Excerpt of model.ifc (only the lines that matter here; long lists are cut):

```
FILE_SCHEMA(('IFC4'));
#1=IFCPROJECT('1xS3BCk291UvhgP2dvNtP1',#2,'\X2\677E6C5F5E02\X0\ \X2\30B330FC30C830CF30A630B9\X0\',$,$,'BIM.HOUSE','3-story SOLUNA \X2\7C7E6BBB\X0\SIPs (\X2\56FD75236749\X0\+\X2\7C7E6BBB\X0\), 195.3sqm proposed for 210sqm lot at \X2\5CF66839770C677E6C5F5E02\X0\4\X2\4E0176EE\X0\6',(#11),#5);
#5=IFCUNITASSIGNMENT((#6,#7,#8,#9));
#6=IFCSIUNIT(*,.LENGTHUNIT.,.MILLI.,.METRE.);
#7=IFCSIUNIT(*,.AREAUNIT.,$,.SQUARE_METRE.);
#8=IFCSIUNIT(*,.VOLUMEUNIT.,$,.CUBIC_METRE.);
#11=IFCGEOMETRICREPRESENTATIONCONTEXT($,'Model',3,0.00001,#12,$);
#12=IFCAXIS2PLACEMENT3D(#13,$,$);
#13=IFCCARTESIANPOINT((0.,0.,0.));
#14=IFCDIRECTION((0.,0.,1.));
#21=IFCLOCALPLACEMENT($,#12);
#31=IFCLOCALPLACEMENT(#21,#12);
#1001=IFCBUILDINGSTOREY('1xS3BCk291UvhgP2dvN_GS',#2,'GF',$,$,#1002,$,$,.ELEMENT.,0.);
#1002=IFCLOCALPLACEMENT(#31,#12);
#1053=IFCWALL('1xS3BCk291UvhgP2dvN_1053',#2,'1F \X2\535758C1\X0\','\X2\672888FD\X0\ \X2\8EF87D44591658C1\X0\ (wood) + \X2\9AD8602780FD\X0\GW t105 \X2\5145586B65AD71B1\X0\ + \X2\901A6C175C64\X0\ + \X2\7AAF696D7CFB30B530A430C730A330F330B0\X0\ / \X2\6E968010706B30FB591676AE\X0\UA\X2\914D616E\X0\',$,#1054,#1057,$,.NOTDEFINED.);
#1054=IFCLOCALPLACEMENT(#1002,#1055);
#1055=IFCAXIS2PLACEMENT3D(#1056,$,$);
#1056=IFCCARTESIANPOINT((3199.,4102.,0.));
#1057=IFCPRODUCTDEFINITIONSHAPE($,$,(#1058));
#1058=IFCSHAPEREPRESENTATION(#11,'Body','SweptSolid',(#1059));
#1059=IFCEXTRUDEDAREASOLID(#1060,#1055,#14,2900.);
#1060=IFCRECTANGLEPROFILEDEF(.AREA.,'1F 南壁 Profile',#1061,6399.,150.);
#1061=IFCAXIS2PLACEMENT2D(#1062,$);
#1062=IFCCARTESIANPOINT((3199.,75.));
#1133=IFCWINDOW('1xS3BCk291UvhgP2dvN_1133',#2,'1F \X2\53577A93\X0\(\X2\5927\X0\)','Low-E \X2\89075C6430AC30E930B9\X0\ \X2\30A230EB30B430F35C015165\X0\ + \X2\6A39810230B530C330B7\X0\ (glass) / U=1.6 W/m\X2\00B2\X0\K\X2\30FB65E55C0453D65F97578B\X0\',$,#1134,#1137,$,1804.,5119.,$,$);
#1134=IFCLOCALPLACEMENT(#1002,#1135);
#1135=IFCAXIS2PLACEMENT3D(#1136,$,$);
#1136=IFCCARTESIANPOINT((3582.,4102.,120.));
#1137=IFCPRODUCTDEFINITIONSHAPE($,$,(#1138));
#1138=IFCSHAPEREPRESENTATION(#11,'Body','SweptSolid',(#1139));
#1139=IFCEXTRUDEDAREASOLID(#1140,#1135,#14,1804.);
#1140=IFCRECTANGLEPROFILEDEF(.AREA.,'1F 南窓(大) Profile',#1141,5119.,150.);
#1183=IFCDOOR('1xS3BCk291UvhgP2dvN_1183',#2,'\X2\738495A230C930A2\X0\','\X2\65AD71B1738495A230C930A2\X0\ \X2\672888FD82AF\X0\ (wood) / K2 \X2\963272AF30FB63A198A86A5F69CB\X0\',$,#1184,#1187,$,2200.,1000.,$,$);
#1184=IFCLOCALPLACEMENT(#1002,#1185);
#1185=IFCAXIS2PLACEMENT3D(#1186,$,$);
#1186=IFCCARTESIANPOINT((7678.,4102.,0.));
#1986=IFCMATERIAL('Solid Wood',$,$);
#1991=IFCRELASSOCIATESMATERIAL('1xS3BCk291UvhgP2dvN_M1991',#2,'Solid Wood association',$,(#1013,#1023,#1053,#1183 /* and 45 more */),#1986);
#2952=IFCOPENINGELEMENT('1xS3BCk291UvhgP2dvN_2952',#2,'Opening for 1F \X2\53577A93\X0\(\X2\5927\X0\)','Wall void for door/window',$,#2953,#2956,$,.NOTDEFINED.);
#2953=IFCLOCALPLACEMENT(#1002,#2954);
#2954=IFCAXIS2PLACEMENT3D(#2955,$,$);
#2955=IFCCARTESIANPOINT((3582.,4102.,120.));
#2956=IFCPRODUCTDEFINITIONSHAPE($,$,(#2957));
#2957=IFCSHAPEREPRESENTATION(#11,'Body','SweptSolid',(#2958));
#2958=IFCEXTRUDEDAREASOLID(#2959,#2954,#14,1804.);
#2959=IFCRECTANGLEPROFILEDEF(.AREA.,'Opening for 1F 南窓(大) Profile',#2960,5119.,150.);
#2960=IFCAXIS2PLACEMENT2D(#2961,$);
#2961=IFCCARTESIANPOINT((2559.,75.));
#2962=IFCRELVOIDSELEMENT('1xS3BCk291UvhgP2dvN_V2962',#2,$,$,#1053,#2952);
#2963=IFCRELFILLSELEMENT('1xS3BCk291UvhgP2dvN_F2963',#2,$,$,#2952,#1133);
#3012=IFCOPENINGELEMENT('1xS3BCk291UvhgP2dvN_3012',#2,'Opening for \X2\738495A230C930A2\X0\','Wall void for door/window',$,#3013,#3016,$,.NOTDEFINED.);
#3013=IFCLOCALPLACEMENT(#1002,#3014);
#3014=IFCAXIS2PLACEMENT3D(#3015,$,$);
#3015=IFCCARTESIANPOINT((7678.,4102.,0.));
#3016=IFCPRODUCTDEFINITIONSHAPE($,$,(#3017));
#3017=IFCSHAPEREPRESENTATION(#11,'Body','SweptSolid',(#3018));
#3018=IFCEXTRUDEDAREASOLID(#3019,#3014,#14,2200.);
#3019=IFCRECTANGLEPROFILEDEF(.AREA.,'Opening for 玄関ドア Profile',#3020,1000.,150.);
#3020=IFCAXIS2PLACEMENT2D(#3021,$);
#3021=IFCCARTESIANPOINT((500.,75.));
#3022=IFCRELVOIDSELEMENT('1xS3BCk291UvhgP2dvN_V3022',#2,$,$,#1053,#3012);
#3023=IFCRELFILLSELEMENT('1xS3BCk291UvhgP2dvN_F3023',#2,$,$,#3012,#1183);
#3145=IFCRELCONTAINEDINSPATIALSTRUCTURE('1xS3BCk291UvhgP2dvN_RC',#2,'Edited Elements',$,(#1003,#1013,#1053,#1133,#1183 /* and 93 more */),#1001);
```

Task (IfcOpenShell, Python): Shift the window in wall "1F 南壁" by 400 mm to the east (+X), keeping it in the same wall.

```python
import ifcopenshell
import ifcopenshell.api.geometry
import ifcopenshell.util.placement
import ifcopenshell.util.unit

model = ifcopenshell.open("model.ifc")
unit_scale = ifcopenshell.util.unit.calculate_unit_scale(model)

window = model.by_guid("1xS3BCk291UvhgP2dvN_1133")
opening = window.FillsVoids[0].RelatingOpeningElement
wall = opening.VoidsElements[0].RelatingBuildingElement

wall_matrix = ifcopenshell.util.placement.get_local_placement(wall.ObjectPlacement)
shift = wall_matrix[:3, 0] * 0.4 / unit_scale
before = ifcopenshell.util.placement.get_local_placement(window.ObjectPlacement)[:3, 3].copy()

# The window is not placed relative to its opening, so move both.
for product in (opening, window):
    matrix = ifcopenshell.util.placement.get_local_placement(product.ObjectPlacement)
    matrix[:3, 3] += shift
    ifcopenshell.api.geometry.edit_object_placement(model, product=product, matrix=matrix, is_si=False)

after = ifcopenshell.util.placement.get_local_placement(window.ObjectPlacement)[:3, 3]
print("window moved by", (after - before).round(3) + 0.0)

model.write("model_rev.ifc")
```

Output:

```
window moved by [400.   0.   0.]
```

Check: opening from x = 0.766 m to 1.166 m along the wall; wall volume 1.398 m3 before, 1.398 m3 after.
